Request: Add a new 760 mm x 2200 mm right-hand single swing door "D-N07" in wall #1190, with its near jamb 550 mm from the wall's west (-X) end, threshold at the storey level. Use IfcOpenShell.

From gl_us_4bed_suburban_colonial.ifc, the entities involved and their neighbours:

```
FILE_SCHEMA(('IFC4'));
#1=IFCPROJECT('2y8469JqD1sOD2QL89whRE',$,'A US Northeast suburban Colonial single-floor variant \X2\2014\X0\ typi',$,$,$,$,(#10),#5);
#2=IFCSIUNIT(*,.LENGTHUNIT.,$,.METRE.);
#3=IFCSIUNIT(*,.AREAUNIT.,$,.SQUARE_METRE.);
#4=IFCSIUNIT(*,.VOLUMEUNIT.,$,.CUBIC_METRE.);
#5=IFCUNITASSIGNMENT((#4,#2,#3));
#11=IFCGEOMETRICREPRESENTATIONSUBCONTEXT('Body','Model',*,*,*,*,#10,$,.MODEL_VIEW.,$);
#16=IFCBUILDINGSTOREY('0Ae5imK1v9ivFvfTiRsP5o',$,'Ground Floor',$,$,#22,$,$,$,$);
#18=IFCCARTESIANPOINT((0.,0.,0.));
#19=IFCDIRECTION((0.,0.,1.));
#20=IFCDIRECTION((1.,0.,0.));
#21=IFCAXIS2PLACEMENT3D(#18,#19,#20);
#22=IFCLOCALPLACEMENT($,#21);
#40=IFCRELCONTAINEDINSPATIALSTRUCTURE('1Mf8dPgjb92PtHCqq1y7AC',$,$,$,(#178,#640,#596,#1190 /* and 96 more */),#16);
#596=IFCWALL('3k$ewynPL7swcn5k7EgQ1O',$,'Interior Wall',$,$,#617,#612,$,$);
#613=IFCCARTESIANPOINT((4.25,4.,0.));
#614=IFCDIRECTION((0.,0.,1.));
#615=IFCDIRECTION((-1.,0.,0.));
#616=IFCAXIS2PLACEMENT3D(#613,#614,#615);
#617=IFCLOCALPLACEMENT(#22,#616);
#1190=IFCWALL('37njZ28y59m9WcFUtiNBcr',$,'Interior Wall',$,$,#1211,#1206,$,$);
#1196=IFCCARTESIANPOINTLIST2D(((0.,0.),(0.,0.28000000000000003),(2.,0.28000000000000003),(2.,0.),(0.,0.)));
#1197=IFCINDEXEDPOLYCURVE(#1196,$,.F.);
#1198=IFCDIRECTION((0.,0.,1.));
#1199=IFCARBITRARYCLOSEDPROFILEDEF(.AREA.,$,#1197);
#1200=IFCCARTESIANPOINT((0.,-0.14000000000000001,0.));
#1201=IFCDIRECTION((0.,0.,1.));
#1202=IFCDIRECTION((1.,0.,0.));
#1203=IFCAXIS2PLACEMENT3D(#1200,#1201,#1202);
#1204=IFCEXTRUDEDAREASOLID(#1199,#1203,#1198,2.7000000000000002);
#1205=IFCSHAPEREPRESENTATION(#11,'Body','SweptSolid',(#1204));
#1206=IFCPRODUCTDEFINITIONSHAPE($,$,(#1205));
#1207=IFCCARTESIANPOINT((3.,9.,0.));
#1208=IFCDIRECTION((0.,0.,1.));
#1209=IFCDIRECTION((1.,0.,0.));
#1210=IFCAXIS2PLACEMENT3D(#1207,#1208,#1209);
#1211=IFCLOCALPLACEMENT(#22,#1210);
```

```python
import numpy as np
import ifcopenshell
import ifcopenshell.api.feature
import ifcopenshell.api.geometry
import ifcopenshell.api.root
import ifcopenshell.api.spatial
import ifcopenshell.geom
import ifcopenshell.util.element
import ifcopenshell.util.placement
import ifcopenshell.util.representation
import ifcopenshell.util.shape
import ifcopenshell.util.unit

model = ifcopenshell.open("gl_us_4bed_suburban_colonial.ifc")
unit_scale = ifcopenshell.util.unit.calculate_unit_scale(model)
settings = ifcopenshell.geom.settings()


def volume(element):
    """Net volume in cubic metres, openings subtracted."""
    shape = ifcopenshell.geom.create_shape(settings, element)
    return ifcopenshell.util.shape.get_volume(shape.geometry)


wall = model.by_guid("37njZ28y59m9WcFUtiNBcr")
storey = ifcopenshell.util.element.get_container(wall, ifc_class="IfcBuildingStorey")
context = ifcopenshell.util.representation.get_context(model, "Model", "Body", "MODEL_VIEW")
before = volume(wall)

width, height, from_end, sill = 0.76, 2.2, 0.55, 0.0  # metres

# The wall runs along its own X axis, and the end named is its -X end.
wall_shape = ifcopenshell.geom.create_shape(settings, wall)
x, y, z = ifcopenshell.util.shape.get_vertices(wall_shape.geometry).T
start = x.min() + from_end
face, thickness = float(y.min()), float(y.max() - y.min())
wall_matrix = ifcopenshell.util.placement.get_local_placement(wall.ObjectPlacement)
level = ifcopenshell.util.placement.get_local_placement(storey.ObjectPlacement)[2, 3]


def in_wall(x, y):
    """Placement at x, y metres in the wall's axes, at sill height."""
    matrix = wall_matrix.copy()
    matrix[:, 3] = wall_matrix @ np.array([x / unit_scale, y / unit_scale, 0.0, 1.0])
    matrix[2, 3] = level + sill / unit_scale
    return matrix


# Opening: a box that overshoots both wall faces by 50 mm.
opening = ifcopenshell.api.root.create_entity(model, ifc_class="IfcOpeningElement", predefined_type="OPENING")
box = ifcopenshell.api.geometry.add_wall_representation(
    model, context=context, length=width, height=height, thickness=thickness + 0.1
)
ifcopenshell.api.geometry.assign_representation(model, product=opening, representation=box)
ifcopenshell.api.geometry.edit_object_placement(model, product=opening, matrix=in_wall(start, face - 0.05), is_si=False)
ifcopenshell.api.feature.add_feature(model, feature=opening, element=wall)

door = ifcopenshell.api.root.create_entity(model, ifc_class="IfcDoor", name="D-N07", predefined_type="DOOR")
door.OverallWidth, door.OverallHeight = width / unit_scale, height / unit_scale
door.OperationType = "SINGLE_SWING_RIGHT"
body = ifcopenshell.api.geometry.add_door_representation(
    model,
    context=context,
    overall_width=door.OverallWidth,
    overall_height=door.OverallHeight,
    operation_type="SINGLE_SWING_RIGHT",
    lining_properties={"LiningDepth": thickness / unit_scale, "ThresholdDepth": thickness / unit_scale},
)
ifcopenshell.api.geometry.assign_representation(model, product=door, representation=body)
ifcopenshell.api.spatial.assign_container(model, products=[door], relating_structure=storey)
ifcopenshell.api.feature.add_filling(model, opening=opening, element=door)

# The lining spans the wall, so the door starts at the wall face.
ifcopenshell.api.geometry.edit_object_placement(model, product=door, matrix=in_wall(start, face), is_si=False)

after = volume(wall)

print(f"wall volume {before:.3f} -> {after:.3f} m3")

model.write("gl_us_4bed_suburban_colonial_updated.ifc")
```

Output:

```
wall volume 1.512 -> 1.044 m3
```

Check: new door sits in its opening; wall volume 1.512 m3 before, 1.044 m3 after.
